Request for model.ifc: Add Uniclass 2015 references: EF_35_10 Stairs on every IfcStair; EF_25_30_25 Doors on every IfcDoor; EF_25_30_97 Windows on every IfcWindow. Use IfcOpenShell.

First a look at what the model holds.

```python
import ifcopenshell

model = ifcopenshell.open("model.ifc")
print(model.schema)
print("classifications:", [c.Name for c in model.by_type("IfcClassification")])
for ifc_class in ("IfcDoor", "IfcRoof", "IfcStair", "IfcWall", "IfcWindow"):
    print(ifc_class, len(model.by_type(ifc_class)))
```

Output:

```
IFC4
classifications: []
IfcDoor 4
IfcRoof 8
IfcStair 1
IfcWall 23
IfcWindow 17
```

```python
import ifcopenshell
import ifcopenshell.api.classification

model = ifcopenshell.open("model.ifc")

system = ifcopenshell.api.classification.add_classification(model, classification="Uniclass 2015")

codes = {
    "IfcStair": ("EF_35_10", "Stairs"),
    "IfcDoor": ("EF_25_30_25", "Doors"),
    "IfcWindow": ("EF_25_30_97", "Windows"),
}
for ifc_class, (code, name) in codes.items():
    products = model.by_type(ifc_class)
    ifcopenshell.api.classification.add_reference(
        model, products=products, classification=system, identification=code, name=name
    )
    print(code, len(products))

model.write("model_edited.ifc")
```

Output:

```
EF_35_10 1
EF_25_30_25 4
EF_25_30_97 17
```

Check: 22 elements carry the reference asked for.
